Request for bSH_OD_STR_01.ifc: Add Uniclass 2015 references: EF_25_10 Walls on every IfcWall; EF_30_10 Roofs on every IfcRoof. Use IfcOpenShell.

First a look at what the model holds.

```python
import ifcopenshell

model = ifcopenshell.open("bSH_OD_STR_01.ifc")
print(model.schema)
print("classifications:", [c.Name for c in model.by_type("IfcClassification")])
for ifc_class in ("IfcDoor", "IfcRoof", "IfcStair", "IfcWall", "IfcWindow"):
    print(ifc_class, len(model.by_type(ifc_class)))
```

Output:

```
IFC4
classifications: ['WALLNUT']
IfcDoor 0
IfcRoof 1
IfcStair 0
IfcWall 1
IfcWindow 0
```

```python
import ifcopenshell
import ifcopenshell.api.classification

model = ifcopenshell.open("bSH_OD_STR_01.ifc")

system = ifcopenshell.api.classification.add_classification(model, classification="Uniclass 2015")

codes = {
    "IfcWall": ("EF_25_10", "Walls"),
    "IfcRoof": ("EF_30_10", "Roofs"),
}
for ifc_class, (code, name) in codes.items():
    products = model.by_type(ifc_class)
    ifcopenshell.api.classification.add_reference(
        model, products=products, classification=system, identification=code, name=name
    )
    print(code, len(products))

model.write("bSH_OD_STR_01_edited.ifc")
```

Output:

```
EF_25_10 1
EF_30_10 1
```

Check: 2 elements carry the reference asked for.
